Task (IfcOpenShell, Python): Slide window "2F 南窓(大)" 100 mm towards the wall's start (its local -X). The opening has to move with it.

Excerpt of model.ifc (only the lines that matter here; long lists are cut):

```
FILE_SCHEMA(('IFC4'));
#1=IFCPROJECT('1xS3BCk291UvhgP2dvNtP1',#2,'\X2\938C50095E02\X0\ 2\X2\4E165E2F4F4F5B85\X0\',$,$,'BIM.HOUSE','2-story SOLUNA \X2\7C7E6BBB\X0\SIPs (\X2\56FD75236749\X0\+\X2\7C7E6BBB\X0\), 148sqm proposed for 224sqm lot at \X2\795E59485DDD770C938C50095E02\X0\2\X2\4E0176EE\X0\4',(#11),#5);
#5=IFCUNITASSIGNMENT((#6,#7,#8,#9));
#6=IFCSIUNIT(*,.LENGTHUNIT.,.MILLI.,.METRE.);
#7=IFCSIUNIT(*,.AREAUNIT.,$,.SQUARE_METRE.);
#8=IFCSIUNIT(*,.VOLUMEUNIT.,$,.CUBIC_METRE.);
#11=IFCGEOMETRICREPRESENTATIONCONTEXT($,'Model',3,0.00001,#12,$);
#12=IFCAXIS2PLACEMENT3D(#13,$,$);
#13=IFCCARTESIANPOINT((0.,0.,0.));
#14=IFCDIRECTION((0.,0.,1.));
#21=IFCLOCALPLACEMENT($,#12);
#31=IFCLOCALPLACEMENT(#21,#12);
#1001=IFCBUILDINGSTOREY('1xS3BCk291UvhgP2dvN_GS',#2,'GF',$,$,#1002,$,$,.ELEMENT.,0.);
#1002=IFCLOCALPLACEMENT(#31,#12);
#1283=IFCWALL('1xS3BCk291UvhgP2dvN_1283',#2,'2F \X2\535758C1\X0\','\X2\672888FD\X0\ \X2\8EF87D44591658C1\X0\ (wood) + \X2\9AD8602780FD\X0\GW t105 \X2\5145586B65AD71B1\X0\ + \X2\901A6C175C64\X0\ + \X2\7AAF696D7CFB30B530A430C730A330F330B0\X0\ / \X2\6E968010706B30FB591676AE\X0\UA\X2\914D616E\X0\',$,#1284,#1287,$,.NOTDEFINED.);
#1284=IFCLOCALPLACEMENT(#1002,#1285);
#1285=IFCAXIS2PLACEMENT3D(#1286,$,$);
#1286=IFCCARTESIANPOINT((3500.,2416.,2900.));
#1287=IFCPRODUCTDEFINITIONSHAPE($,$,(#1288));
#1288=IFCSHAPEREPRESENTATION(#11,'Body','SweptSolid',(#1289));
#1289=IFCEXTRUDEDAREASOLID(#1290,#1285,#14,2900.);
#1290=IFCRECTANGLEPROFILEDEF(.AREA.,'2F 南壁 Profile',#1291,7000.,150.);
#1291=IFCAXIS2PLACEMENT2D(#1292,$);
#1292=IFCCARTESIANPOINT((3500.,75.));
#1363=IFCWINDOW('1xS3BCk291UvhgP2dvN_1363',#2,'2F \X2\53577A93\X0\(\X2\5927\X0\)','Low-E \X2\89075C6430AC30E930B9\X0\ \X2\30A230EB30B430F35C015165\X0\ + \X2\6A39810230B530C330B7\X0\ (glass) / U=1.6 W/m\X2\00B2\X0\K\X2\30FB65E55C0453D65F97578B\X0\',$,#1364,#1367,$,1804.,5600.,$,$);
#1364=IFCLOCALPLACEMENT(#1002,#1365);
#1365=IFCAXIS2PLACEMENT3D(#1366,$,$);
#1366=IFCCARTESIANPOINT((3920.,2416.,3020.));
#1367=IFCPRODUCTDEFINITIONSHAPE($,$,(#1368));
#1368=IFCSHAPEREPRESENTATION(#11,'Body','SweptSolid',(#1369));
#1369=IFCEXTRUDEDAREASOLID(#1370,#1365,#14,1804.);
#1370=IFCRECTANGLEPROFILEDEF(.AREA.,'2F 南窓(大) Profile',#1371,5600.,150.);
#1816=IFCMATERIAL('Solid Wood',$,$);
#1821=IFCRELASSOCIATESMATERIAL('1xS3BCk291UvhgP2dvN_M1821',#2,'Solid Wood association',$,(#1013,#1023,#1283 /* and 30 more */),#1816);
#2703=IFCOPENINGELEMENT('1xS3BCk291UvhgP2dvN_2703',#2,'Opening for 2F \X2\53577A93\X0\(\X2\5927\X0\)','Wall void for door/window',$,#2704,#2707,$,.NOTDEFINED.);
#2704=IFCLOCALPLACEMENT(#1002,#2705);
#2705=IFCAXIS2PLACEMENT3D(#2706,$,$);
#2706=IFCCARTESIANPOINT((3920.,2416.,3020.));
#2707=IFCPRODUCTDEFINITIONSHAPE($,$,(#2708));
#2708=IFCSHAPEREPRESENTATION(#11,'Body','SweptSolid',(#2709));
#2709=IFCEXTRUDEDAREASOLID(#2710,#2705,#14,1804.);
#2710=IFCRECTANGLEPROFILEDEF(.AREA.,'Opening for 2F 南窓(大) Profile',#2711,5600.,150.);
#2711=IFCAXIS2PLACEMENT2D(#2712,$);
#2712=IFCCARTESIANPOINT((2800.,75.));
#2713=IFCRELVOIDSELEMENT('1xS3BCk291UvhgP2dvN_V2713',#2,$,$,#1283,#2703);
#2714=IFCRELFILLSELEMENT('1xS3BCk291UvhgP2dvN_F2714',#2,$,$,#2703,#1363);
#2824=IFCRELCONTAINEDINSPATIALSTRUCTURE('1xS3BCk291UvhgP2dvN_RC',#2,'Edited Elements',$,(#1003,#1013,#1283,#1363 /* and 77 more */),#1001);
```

```python
import ifcopenshell
import ifcopenshell.api.geometry
import ifcopenshell.util.placement

model = ifcopenshell.open("model.ifc")

window = model.by_guid("1xS3BCk291UvhgP2dvN_1363")
opening = window.FillsVoids[0].RelatingOpeningElement
wall = opening.VoidsElements[0].RelatingBuildingElement

wall_matrix = ifcopenshell.util.placement.get_local_placement(wall.ObjectPlacement)
shift = wall_matrix[:3, 0] * -100.0
before = ifcopenshell.util.placement.get_local_placement(window.ObjectPlacement)[:3, 3].copy()

# The window is not placed relative to its opening, so move both.
for product in (opening, window):
    matrix = ifcopenshell.util.placement.get_local_placement(product.ObjectPlacement)
    matrix[:3, 3] += shift
    ifcopenshell.api.geometry.edit_object_placement(model, product=product, matrix=matrix, is_si=False)

after = ifcopenshell.util.placement.get_local_placement(window.ObjectPlacement)[:3, 3]
print("window moved by", (after - before).round(3) + 0.0)

model.write("model_updated.ifc")
```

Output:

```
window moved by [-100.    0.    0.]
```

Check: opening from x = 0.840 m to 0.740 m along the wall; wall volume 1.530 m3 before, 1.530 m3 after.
